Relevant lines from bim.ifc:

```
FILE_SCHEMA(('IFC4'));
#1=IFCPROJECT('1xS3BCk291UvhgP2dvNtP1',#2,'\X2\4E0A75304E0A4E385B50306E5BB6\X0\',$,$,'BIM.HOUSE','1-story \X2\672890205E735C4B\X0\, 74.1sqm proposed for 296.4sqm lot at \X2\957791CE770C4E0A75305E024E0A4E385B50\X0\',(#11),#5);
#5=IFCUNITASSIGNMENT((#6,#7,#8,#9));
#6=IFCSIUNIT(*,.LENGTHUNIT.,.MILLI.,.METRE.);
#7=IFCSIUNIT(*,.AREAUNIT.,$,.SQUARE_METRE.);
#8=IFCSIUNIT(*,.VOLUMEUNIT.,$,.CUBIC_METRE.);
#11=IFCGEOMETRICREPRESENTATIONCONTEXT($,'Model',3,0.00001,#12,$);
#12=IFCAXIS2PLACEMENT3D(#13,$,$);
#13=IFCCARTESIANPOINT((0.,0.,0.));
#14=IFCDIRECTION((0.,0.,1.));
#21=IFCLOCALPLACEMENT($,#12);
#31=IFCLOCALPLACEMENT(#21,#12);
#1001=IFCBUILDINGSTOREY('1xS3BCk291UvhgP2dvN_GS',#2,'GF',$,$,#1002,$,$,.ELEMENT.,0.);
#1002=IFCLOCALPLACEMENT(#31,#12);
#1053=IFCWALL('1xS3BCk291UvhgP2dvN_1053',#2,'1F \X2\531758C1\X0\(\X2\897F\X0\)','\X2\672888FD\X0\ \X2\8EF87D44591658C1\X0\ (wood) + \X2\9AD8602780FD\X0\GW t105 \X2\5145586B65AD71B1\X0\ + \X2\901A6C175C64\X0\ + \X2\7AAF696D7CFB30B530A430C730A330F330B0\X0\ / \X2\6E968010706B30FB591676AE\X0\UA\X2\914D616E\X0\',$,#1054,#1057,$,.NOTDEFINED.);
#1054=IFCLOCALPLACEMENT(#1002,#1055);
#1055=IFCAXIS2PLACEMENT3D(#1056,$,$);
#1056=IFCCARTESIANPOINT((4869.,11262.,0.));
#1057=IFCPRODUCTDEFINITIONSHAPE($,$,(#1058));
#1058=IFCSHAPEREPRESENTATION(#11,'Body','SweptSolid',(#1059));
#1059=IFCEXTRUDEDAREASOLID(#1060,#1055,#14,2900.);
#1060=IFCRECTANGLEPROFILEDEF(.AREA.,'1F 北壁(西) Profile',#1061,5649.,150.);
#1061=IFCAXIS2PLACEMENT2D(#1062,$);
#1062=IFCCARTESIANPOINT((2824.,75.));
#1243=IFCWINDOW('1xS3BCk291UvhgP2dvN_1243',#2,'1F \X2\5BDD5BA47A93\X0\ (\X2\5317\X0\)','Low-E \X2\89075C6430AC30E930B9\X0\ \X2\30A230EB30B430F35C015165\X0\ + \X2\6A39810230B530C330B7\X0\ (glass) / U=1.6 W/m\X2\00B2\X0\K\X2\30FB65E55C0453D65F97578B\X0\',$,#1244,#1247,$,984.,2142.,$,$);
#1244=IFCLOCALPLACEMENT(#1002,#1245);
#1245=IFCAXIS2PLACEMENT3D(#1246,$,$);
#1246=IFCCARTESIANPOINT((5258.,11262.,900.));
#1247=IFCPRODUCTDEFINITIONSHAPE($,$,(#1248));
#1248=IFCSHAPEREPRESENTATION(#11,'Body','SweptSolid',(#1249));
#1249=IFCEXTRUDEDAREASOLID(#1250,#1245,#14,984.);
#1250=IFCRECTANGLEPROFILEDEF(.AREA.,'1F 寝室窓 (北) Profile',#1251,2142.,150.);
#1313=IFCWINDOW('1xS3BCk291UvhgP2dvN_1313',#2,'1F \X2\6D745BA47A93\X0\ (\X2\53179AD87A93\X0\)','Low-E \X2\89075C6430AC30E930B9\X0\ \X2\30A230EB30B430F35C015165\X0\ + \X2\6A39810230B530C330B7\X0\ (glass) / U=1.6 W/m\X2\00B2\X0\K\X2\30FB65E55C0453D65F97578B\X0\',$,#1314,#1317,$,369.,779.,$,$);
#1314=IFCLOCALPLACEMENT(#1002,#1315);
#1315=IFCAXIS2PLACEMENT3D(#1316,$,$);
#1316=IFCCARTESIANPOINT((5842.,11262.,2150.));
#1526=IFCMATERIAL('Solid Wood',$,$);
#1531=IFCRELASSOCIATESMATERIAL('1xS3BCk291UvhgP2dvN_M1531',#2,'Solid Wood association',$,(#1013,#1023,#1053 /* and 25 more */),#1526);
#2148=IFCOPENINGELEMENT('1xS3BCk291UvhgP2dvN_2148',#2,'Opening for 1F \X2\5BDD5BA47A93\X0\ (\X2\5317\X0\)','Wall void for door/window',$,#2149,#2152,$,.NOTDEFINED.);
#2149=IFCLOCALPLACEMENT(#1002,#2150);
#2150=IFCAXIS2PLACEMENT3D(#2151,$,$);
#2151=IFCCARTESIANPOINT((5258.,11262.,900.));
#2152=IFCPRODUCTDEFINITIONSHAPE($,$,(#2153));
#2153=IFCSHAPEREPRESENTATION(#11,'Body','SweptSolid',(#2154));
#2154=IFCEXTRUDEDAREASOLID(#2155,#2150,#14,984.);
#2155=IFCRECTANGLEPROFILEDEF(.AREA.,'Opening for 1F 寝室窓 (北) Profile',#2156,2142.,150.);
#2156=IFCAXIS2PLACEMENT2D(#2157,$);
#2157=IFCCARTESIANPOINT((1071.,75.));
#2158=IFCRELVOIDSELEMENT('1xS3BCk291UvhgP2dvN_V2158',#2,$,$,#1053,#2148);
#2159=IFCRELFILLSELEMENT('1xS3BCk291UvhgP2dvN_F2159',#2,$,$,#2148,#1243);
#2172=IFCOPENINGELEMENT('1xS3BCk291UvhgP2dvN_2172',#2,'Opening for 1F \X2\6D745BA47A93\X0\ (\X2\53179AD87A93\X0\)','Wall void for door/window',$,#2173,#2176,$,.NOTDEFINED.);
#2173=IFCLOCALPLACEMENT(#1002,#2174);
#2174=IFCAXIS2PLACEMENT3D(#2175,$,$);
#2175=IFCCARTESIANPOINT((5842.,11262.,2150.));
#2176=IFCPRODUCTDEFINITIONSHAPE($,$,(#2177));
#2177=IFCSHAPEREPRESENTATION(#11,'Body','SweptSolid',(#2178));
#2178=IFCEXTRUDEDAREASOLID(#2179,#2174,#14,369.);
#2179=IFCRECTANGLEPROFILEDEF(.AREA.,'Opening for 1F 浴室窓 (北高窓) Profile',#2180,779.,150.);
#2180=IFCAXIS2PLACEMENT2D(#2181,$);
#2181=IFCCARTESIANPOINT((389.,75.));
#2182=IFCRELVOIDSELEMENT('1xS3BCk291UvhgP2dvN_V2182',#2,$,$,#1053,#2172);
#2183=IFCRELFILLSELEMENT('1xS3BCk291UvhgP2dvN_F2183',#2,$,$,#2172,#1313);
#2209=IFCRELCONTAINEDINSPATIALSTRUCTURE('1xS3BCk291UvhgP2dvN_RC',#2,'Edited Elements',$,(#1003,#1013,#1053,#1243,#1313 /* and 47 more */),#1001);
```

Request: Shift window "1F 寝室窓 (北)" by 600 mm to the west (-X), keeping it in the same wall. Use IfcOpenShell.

```python
import ifcopenshell
import ifcopenshell.api.geometry
import ifcopenshell.util.placement
import ifcopenshell.util.unit

model = ifcopenshell.open("bim.ifc")
unit_scale = ifcopenshell.util.unit.calculate_unit_scale(model)

window = model.by_id(1243)
opening = window.FillsVoids[0].RelatingOpeningElement
wall = opening.VoidsElements[0].RelatingBuildingElement

wall_matrix = ifcopenshell.util.placement.get_local_placement(wall.ObjectPlacement)
shift = wall_matrix[:3, 0] * -0.6 / unit_scale
before = ifcopenshell.util.placement.get_local_placement(window.ObjectPlacement)[:3, 3].copy()

# The window is not placed relative to its opening, so move both.
for product in (opening, window):
    matrix = ifcopenshell.util.placement.get_local_placement(product.ObjectPlacement)
    matrix[:3, 3] += shift
    ifcopenshell.api.geometry.edit_object_placement(model, product=product, matrix=matrix, is_si=False)

after = ifcopenshell.util.placement.get_local_placement(window.ObjectPlacement)[:3, 3]
print("window moved by", (after - before).round(3) + 0.0)

model.write("bim_edited.ifc")
```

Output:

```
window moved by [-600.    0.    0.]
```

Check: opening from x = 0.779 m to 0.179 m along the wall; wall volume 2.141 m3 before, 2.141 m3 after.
